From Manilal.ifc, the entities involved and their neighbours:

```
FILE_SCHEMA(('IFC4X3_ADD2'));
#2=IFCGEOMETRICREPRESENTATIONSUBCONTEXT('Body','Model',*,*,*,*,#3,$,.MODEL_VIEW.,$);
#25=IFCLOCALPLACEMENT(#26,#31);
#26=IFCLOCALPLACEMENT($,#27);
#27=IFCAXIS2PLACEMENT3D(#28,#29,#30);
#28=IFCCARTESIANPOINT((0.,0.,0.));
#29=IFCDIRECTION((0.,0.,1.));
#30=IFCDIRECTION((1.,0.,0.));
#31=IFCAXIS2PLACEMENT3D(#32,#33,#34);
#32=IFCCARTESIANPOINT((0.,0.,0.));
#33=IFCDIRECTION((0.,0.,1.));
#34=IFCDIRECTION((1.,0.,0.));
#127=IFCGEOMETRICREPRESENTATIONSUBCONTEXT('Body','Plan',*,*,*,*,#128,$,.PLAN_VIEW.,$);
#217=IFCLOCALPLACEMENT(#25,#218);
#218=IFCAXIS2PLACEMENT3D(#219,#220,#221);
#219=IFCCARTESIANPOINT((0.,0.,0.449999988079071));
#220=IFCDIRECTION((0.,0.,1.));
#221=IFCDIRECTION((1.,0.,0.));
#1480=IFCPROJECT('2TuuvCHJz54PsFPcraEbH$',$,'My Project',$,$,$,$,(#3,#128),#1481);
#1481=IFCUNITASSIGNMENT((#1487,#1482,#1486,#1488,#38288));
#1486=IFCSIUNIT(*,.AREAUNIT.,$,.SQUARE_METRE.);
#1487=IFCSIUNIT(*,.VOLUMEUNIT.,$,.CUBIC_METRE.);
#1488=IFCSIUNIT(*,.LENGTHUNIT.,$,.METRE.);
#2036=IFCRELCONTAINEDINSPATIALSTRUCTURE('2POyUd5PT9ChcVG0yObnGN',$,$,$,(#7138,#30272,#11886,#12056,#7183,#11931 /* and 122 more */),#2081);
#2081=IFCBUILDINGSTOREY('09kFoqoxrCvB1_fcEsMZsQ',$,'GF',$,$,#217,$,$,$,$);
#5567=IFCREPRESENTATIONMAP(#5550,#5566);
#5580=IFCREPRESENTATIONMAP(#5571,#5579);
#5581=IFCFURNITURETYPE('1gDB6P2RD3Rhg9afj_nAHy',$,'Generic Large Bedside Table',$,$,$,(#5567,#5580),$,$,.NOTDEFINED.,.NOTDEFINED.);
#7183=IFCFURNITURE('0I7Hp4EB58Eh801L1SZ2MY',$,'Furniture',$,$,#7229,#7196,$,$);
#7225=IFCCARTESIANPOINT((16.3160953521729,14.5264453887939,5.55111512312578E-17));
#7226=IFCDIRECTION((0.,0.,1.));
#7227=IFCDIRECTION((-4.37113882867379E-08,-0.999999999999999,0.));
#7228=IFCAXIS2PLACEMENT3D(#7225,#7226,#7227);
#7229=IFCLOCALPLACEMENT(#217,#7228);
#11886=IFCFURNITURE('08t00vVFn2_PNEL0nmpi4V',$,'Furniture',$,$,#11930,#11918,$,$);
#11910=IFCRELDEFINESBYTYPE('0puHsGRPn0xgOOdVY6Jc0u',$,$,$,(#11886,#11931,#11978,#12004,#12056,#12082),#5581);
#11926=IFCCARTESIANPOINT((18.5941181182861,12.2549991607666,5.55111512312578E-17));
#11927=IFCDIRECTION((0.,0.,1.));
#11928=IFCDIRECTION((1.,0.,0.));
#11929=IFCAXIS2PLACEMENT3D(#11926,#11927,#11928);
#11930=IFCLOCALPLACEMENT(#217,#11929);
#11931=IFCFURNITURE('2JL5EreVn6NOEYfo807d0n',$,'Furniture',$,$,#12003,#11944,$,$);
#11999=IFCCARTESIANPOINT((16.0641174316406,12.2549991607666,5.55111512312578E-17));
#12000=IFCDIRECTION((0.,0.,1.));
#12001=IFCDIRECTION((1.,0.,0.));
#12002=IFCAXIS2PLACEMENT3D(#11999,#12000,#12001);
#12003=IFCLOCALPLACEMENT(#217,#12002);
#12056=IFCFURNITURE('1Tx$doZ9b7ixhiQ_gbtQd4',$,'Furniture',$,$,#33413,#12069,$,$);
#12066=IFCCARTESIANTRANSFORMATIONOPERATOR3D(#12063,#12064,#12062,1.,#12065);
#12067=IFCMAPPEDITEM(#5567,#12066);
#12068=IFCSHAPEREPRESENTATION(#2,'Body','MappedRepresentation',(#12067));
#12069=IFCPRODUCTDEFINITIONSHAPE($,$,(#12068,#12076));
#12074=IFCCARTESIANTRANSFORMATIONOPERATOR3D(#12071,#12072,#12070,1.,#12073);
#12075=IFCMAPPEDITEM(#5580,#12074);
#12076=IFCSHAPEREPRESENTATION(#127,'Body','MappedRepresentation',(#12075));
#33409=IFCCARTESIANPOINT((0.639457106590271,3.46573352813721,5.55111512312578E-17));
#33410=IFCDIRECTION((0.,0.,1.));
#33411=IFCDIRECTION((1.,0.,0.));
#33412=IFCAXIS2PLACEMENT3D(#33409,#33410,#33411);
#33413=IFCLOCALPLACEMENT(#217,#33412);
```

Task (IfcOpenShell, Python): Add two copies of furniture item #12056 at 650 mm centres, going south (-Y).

```python
import numpy as np
import ifcopenshell
import ifcopenshell.api.geometry
import ifcopenshell.api.root
import ifcopenshell.util.element
import ifcopenshell.util.placement
import ifcopenshell.util.unit

model = ifcopenshell.open("Manilal.ifc")
unit_scale = ifcopenshell.util.unit.calculate_unit_scale(model)

source = model.by_guid("1Tx$doZ9b7ixhiQ_gbtQd4")
base = ifcopenshell.util.placement.get_local_placement(source.ObjectPlacement)
step = np.array([0.0, -1.0, 0.0]) * 0.65 / unit_scale

for i in range(1, 3):
    copy = ifcopenshell.api.root.copy_class(model, product=source)
    copy.Representation = ifcopenshell.util.element.copy_deep(
        model, source.Representation, exclude=["IfcGeometricRepresentationContext", "IfcRepresentationMap"]
    )
    matrix = base.copy()
    matrix[:3, 3] += i * step
    print("added at", matrix[:3, 3].round(3) + 0.0)
    ifcopenshell.api.geometry.edit_object_placement(model, product=copy, matrix=matrix, is_si=False)

model.write("Manilal_v2.ifc")
```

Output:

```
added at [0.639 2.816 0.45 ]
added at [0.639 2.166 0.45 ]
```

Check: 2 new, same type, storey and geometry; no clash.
